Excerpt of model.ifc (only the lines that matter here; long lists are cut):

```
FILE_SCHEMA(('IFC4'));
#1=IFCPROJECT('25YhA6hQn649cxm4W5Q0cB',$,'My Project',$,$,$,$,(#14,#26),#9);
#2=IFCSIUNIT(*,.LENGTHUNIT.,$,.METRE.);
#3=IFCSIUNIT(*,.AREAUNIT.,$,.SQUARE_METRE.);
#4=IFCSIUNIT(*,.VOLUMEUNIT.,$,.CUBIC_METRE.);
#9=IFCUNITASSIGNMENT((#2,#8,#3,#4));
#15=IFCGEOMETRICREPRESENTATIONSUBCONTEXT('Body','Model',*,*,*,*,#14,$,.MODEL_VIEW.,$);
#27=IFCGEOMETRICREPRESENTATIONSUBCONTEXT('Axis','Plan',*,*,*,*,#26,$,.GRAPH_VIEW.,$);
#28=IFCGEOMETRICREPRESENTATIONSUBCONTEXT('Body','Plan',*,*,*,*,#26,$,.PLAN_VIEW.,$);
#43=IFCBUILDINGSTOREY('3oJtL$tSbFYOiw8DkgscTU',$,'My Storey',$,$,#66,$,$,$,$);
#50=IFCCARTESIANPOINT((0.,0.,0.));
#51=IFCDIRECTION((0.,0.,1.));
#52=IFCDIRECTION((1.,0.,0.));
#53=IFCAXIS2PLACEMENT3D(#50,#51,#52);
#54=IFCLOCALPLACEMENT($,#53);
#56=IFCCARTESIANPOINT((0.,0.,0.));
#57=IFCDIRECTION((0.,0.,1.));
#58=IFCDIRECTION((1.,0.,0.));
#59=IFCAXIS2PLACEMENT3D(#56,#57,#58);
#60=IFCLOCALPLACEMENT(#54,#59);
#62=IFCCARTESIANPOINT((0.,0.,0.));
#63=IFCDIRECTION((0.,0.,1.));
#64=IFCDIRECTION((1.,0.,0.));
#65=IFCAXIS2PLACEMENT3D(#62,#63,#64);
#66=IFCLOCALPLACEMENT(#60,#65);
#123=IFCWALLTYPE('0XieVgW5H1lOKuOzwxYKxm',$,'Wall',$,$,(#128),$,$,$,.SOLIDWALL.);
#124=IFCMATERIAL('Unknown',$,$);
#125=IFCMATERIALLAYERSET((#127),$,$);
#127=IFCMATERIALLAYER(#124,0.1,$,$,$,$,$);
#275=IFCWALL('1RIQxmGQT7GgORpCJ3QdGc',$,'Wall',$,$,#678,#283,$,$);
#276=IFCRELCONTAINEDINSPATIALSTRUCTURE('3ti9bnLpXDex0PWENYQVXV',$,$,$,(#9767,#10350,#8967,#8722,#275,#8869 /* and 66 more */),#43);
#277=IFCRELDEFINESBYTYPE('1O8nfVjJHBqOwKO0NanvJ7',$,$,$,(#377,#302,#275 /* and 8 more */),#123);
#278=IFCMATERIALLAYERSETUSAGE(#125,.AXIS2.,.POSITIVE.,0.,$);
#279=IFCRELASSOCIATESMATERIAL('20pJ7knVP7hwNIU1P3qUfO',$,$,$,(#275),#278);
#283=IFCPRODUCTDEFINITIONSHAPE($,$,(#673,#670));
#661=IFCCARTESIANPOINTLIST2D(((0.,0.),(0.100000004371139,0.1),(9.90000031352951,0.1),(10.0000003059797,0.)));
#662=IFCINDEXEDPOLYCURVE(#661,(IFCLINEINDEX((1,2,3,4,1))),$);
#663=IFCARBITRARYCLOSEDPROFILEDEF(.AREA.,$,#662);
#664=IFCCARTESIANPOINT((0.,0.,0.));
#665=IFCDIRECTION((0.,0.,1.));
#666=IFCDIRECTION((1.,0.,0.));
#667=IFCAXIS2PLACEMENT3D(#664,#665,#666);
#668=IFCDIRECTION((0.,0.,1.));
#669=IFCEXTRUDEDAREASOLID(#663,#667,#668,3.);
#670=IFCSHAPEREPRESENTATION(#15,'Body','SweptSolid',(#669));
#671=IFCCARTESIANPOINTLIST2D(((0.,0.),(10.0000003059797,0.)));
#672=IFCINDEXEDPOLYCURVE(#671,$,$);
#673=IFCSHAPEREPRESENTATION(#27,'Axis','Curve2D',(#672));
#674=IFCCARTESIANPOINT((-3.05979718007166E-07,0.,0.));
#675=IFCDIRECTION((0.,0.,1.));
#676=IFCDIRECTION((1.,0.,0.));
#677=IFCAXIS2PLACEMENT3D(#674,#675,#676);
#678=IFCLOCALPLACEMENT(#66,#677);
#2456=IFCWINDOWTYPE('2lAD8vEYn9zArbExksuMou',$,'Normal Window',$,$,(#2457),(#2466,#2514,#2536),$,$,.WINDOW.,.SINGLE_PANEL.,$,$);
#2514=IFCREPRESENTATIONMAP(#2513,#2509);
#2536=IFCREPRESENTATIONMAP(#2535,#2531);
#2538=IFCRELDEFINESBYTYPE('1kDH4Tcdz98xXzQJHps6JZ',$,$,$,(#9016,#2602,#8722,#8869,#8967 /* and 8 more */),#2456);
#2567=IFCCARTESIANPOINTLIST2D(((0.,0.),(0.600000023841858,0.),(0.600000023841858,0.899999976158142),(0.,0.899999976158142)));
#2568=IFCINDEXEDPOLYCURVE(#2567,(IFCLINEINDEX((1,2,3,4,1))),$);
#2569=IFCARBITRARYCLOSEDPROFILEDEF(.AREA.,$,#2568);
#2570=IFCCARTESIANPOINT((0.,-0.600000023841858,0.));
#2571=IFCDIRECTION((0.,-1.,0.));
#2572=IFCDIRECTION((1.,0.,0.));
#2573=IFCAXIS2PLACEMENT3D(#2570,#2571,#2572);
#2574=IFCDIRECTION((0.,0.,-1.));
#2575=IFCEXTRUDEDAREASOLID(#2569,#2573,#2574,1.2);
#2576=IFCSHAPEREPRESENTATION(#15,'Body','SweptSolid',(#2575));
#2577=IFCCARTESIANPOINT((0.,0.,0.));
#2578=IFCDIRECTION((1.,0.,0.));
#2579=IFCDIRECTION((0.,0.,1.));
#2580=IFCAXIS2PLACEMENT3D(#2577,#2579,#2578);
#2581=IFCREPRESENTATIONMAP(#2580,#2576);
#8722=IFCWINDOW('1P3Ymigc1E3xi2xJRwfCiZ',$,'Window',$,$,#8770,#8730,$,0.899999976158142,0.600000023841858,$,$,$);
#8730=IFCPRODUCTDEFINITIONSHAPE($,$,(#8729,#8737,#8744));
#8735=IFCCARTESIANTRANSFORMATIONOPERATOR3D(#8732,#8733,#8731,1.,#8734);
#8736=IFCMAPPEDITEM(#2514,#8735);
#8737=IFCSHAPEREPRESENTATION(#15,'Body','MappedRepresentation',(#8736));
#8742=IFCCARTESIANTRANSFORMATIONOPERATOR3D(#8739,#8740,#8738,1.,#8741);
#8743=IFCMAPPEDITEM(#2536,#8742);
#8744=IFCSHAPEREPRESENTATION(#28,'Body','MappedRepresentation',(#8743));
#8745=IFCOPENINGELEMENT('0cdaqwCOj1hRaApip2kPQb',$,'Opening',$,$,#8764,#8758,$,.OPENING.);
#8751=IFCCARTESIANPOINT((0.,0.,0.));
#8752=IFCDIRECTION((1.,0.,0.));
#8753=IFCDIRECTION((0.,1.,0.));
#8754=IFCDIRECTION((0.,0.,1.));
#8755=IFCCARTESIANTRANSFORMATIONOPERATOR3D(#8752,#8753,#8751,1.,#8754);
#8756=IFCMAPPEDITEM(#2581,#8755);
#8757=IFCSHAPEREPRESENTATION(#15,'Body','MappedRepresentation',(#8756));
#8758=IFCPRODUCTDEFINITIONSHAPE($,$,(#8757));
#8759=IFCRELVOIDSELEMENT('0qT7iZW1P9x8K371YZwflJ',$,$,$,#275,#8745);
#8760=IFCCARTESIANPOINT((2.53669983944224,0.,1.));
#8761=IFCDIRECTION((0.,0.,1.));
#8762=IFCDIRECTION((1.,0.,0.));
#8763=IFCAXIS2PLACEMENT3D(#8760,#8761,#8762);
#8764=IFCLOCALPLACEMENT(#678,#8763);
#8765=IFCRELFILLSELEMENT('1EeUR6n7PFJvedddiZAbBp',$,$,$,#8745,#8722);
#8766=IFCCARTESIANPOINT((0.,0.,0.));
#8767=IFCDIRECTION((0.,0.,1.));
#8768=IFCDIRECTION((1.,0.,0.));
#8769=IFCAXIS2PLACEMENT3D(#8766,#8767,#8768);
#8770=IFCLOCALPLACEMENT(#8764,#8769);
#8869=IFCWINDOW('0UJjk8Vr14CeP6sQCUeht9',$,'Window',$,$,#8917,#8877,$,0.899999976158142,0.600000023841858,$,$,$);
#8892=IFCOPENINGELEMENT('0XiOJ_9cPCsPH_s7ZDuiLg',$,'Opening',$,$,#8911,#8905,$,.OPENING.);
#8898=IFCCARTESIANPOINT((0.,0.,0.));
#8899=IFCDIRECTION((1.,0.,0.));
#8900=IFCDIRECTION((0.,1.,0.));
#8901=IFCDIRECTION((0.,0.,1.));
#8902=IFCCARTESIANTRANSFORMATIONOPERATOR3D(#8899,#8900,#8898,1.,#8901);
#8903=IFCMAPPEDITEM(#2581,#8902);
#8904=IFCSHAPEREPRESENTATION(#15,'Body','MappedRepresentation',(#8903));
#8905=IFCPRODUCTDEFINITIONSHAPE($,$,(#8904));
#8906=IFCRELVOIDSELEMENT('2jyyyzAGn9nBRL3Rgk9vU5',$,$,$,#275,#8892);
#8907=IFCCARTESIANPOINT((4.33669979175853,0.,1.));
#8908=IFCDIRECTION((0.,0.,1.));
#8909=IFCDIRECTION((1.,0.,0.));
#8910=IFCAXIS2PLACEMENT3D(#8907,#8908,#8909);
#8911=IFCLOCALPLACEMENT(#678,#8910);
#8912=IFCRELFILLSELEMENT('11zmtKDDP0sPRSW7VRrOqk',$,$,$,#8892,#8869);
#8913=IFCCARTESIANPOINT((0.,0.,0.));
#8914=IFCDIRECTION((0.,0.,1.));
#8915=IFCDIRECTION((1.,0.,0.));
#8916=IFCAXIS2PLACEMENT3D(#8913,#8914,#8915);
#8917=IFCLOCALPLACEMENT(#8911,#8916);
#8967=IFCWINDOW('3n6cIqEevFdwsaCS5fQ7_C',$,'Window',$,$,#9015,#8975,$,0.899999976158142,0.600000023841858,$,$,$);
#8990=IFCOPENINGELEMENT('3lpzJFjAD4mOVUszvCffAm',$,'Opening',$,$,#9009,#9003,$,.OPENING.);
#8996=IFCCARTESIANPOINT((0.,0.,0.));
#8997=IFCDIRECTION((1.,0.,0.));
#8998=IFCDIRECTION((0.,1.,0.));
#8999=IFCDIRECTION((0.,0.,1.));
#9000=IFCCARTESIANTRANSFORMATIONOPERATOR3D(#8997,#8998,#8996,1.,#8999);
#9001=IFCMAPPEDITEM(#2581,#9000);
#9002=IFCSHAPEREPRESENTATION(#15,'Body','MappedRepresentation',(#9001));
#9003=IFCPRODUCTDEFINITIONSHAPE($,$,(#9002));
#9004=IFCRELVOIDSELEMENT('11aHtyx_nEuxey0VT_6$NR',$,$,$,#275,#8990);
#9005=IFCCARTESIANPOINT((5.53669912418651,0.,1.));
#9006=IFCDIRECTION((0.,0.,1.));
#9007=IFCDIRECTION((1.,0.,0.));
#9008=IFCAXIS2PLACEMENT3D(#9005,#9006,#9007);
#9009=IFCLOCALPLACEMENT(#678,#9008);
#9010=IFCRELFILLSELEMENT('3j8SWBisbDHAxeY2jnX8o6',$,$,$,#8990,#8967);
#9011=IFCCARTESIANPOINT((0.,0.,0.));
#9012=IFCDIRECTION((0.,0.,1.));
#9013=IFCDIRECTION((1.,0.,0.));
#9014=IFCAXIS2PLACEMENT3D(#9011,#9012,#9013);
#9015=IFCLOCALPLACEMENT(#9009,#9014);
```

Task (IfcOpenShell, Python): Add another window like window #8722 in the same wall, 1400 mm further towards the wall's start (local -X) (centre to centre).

```python
import ifcopenshell
import ifcopenshell.api.feature
import ifcopenshell.api.geometry
import ifcopenshell.api.root
import ifcopenshell.geom
import ifcopenshell.util.element
import ifcopenshell.util.placement
import ifcopenshell.util.shape

model = ifcopenshell.open("model.ifc")
settings = ifcopenshell.geom.settings()


def volume(element):
    """Net volume in cubic metres, openings subtracted."""
    shape = ifcopenshell.geom.create_shape(settings, element)
    return ifcopenshell.util.shape.get_volume(shape.geometry)


window = model.by_id(8722)
opening = window.FillsVoids[0].RelatingOpeningElement
wall = opening.VoidsElements[0].RelatingBuildingElement
before = volume(wall)
shift = ifcopenshell.util.placement.get_local_placement(wall.ObjectPlacement)[:3, 0] * -1.4

# copy_class copies the void relationship, type, container and properties, but no geometry.
new_opening = ifcopenshell.api.root.copy_class(model, product=opening)
new_opening.Representation = ifcopenshell.util.element.copy_deep(
    model, opening.Representation, exclude=["IfcGeometricRepresentationContext", "IfcRepresentationMap"]
)
new_window = ifcopenshell.api.root.copy_class(model, product=window)
new_window.Representation = ifcopenshell.util.element.copy_deep(
    model, window.Representation, exclude=["IfcGeometricRepresentationContext", "IfcRepresentationMap"]
)
ifcopenshell.api.feature.add_filling(model, opening=new_opening, element=new_window)

for old, new in ((opening, new_opening), (window, new_window)):
    matrix = ifcopenshell.util.placement.get_local_placement(old.ObjectPlacement)
    matrix[:3, 3] += shift
    ifcopenshell.api.geometry.edit_object_placement(model, product=new, matrix=matrix, is_si=False)

after = volume(wall)

print(f"wall volume {before:.3f} -> {after:.3f} m3")

model.write("model_v2.ifc")
```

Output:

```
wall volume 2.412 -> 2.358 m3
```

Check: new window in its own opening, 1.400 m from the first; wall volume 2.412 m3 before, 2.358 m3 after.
